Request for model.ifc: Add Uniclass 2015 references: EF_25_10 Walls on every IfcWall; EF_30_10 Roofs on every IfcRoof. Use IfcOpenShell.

First a look at what the model holds.

```python
import ifcopenshell

model = ifcopenshell.open("model.ifc")
print(model.schema)
print("classifications:", [c.Name for c in model.by_type("IfcClassification")])
for ifc_class in ("IfcDoor", "IfcRoof", "IfcStair", "IfcWall", "IfcWindow"):
    print(ifc_class, len(model.by_type(ifc_class)))
```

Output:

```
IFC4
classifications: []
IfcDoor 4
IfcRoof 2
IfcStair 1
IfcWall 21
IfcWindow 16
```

```python
import ifcopenshell
import ifcopenshell.api.classification

model = ifcopenshell.open("model.ifc")

system = ifcopenshell.api.classification.add_classification(model, classification="Uniclass 2015")

codes = {
    "IfcWall": ("EF_25_10", "Walls"),
    "IfcRoof": ("EF_30_10", "Roofs"),
}
for ifc_class, (code, name) in codes.items():
    products = model.by_type(ifc_class)
    ifcopenshell.api.classification.add_reference(
        model, products=products, classification=system, identification=code, name=name
    )
    print(code, len(products))

model.write("model_v2.ifc")
```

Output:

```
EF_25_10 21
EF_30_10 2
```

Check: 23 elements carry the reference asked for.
